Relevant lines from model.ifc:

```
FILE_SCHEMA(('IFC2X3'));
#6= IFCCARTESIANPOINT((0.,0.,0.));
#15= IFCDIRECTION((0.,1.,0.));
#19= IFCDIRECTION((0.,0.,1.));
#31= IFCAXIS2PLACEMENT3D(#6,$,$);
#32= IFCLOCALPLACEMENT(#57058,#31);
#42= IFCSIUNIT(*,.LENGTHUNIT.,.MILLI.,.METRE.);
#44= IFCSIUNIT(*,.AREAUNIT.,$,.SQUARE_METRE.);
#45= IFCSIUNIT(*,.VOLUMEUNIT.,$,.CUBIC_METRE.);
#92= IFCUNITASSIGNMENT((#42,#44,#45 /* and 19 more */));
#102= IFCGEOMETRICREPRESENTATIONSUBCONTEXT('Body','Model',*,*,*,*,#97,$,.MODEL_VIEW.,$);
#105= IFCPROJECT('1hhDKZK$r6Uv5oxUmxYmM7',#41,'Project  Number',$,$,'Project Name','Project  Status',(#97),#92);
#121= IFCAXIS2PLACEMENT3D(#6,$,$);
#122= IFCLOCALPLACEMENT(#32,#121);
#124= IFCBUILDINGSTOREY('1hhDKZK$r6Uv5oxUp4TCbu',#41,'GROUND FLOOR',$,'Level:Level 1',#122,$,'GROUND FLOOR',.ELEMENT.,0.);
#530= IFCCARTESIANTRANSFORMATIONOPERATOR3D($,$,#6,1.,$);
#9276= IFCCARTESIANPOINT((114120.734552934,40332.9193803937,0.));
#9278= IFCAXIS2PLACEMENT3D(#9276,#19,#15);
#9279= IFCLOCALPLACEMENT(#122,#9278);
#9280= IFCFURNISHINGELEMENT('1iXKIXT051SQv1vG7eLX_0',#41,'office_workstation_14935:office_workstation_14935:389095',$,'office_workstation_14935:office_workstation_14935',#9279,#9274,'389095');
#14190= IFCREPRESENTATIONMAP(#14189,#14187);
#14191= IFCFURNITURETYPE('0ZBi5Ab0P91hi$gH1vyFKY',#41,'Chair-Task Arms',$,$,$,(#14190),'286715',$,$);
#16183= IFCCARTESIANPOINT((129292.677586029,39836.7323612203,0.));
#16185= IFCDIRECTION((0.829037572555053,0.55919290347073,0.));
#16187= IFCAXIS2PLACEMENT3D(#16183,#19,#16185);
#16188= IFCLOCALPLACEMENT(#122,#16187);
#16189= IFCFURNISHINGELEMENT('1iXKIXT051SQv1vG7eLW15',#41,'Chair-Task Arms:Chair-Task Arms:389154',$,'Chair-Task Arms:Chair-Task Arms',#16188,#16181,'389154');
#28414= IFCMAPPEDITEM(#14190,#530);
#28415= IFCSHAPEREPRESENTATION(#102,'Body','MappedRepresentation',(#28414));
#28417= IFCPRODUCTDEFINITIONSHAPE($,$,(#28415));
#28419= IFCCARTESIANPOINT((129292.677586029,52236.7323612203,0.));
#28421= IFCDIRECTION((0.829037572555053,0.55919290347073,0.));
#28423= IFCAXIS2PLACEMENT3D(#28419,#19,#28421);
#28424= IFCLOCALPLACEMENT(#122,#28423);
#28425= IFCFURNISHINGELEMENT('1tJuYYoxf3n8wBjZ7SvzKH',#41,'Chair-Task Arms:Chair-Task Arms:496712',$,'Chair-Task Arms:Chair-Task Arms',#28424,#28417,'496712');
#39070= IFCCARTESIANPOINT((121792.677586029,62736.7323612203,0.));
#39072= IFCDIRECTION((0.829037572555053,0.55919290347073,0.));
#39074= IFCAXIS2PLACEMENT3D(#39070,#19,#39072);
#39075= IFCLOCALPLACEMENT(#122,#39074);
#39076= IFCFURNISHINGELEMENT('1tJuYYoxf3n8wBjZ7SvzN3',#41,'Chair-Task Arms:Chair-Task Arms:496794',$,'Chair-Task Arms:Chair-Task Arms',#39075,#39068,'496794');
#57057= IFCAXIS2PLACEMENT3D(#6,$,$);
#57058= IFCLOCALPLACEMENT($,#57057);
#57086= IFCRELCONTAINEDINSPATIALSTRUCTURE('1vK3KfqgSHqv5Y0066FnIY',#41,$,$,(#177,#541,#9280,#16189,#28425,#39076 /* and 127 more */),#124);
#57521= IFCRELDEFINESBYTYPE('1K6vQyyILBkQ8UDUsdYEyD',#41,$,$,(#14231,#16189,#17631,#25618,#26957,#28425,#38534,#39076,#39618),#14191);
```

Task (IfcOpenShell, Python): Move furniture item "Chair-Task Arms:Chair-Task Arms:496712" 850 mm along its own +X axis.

```python
import ifcopenshell
import ifcopenshell.api.geometry
import ifcopenshell.util.placement
import ifcopenshell.util.unit

model = ifcopenshell.open("model.ifc")
unit_scale = ifcopenshell.util.unit.calculate_unit_scale(model)

item = model.by_guid("1tJuYYoxf3n8wBjZ7SvzKH")
matrix = ifcopenshell.util.placement.get_local_placement(item.ObjectPlacement)
matrix[:3, 3] += matrix[:3, 0] * 0.85 / unit_scale
ifcopenshell.api.geometry.edit_object_placement(model, product=item, matrix=matrix, is_si=False)

print(ifcopenshell.util.placement.get_local_placement(item.ObjectPlacement).round(3) + 0.0)

model.write("model_v2.ifc")
```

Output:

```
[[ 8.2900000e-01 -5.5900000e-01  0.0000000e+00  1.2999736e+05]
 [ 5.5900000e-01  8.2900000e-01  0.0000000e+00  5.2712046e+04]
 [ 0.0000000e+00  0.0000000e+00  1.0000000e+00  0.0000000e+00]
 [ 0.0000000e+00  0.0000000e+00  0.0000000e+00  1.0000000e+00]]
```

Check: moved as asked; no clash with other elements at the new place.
